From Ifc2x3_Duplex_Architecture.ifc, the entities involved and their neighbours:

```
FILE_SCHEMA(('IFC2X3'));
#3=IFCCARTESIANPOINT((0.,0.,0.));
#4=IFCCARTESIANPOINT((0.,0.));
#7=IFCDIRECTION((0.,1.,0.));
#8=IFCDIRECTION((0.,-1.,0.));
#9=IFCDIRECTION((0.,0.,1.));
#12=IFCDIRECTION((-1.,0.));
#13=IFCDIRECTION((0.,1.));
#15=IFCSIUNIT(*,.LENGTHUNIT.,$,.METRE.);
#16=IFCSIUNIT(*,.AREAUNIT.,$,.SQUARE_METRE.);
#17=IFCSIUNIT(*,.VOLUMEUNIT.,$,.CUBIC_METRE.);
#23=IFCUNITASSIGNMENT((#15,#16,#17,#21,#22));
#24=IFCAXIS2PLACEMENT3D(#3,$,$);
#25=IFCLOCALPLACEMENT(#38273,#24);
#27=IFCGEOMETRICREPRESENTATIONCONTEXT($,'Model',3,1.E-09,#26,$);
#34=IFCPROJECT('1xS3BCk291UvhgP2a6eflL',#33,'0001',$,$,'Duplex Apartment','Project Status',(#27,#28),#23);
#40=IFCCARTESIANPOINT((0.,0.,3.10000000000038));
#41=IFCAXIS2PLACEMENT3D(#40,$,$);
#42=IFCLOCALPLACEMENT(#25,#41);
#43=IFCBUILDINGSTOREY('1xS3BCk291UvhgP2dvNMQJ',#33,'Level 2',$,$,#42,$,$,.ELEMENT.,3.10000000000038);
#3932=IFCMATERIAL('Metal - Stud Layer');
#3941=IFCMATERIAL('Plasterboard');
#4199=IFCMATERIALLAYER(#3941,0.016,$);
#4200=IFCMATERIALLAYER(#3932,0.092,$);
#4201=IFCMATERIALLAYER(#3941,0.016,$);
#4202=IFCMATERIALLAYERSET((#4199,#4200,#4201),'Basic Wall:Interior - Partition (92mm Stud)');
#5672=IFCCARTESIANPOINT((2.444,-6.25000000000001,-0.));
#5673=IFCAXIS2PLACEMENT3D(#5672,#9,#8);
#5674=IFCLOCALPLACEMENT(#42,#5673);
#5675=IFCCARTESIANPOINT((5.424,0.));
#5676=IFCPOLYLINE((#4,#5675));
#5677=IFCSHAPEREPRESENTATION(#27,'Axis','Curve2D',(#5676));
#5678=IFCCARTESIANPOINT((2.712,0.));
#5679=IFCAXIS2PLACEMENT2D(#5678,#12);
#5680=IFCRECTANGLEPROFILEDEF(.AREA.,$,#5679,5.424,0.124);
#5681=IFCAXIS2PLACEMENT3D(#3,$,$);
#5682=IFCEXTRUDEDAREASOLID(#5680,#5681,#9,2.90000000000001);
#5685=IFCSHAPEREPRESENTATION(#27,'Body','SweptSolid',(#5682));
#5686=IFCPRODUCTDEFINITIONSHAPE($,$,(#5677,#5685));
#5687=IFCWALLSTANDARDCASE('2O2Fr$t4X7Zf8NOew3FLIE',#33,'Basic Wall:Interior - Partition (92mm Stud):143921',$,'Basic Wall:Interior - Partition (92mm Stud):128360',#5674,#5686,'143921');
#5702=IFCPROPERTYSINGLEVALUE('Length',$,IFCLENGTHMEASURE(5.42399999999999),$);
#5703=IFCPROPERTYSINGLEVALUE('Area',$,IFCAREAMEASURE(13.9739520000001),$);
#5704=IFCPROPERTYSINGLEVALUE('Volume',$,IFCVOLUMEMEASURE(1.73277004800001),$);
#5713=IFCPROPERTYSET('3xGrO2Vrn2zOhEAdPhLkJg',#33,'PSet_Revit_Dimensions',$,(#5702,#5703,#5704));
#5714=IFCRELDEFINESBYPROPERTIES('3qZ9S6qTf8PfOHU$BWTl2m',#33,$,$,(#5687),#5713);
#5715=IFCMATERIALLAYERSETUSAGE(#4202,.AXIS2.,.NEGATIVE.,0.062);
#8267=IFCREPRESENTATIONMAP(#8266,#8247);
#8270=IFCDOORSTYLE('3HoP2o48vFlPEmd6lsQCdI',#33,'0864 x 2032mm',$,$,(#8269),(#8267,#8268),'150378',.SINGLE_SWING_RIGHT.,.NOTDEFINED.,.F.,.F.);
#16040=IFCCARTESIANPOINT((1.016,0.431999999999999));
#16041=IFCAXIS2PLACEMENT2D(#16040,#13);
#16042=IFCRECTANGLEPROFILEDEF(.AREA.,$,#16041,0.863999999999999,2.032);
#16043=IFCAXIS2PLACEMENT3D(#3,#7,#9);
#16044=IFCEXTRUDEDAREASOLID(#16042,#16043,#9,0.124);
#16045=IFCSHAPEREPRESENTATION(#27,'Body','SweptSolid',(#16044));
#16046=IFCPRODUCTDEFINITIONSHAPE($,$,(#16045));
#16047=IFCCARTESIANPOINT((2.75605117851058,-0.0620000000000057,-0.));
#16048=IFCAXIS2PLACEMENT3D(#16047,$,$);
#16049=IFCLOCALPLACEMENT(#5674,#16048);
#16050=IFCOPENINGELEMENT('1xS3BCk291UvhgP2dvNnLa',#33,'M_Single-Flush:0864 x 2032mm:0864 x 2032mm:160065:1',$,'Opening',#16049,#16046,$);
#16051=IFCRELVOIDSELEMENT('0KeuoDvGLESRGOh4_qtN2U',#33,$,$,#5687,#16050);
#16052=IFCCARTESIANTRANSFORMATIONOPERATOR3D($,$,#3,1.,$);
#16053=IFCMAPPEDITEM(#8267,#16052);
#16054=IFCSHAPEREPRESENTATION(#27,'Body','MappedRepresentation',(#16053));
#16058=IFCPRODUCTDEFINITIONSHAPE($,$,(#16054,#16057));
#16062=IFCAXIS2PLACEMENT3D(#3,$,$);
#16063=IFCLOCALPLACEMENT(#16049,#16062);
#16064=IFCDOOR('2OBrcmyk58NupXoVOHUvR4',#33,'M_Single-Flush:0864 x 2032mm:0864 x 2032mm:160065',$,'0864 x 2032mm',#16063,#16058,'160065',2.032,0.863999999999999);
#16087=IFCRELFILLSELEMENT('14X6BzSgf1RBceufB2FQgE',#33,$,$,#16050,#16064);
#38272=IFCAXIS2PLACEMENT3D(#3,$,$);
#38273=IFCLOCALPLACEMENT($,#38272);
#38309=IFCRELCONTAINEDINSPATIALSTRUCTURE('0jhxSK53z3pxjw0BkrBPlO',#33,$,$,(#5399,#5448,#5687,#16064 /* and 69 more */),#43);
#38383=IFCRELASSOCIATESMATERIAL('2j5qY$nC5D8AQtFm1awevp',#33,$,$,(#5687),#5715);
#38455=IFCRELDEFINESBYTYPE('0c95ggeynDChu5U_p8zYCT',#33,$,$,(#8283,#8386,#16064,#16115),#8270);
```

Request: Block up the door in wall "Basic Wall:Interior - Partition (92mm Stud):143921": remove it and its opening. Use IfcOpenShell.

```python
import ifcopenshell
import ifcopenshell.api.feature
import ifcopenshell.api.pset
import ifcopenshell.api.root
import ifcopenshell.geom
import ifcopenshell.util.element
import ifcopenshell.util.shape
import ifcopenshell.util.unit

model = ifcopenshell.open("Ifc2x3_Duplex_Architecture.ifc")
area_scale = ifcopenshell.util.unit.calculate_unit_scale(model, "AREAUNIT")
volume_scale = ifcopenshell.util.unit.calculate_unit_scale(model, "VOLUMEUNIT")
settings = ifcopenshell.geom.settings()


def volume(element):
    """Net volume in cubic metres, openings subtracted."""
    shape = ifcopenshell.geom.create_shape(settings, element)
    return ifcopenshell.util.shape.get_volume(shape.geometry)


door = model.by_id(16064)
opening = door.FillsVoids[0].RelatingOpeningElement
wall = opening.VoidsElements[0].RelatingBuildingElement
before = volume(wall)

ifcopenshell.api.root.remove_product(model, product=door)
ifcopenshell.api.feature.remove_feature(model, feature=opening)

after = volume(wall)
thickness = 0.124  # wall thickness in metres

# Update the wall's stored quantities.
pset = model.by_id(ifcopenshell.util.element.get_pset(wall, "PSet_Revit_Dimensions", should_inherit=False)["id"])
ifcopenshell.api.pset.edit_pset(model, pset=pset, properties={
    "Area": model.create_entity("IfcAreaMeasure", after / thickness / area_scale),
    "Volume": model.create_entity("IfcVolumeMeasure", after / volume_scale),
})

print(f"wall volume {before:.3f} -> {after:.3f} m3")

model.write("Ifc2x3_Duplex_Architecture_edited.ifc")
```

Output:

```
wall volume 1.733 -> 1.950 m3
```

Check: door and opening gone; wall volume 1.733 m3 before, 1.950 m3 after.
